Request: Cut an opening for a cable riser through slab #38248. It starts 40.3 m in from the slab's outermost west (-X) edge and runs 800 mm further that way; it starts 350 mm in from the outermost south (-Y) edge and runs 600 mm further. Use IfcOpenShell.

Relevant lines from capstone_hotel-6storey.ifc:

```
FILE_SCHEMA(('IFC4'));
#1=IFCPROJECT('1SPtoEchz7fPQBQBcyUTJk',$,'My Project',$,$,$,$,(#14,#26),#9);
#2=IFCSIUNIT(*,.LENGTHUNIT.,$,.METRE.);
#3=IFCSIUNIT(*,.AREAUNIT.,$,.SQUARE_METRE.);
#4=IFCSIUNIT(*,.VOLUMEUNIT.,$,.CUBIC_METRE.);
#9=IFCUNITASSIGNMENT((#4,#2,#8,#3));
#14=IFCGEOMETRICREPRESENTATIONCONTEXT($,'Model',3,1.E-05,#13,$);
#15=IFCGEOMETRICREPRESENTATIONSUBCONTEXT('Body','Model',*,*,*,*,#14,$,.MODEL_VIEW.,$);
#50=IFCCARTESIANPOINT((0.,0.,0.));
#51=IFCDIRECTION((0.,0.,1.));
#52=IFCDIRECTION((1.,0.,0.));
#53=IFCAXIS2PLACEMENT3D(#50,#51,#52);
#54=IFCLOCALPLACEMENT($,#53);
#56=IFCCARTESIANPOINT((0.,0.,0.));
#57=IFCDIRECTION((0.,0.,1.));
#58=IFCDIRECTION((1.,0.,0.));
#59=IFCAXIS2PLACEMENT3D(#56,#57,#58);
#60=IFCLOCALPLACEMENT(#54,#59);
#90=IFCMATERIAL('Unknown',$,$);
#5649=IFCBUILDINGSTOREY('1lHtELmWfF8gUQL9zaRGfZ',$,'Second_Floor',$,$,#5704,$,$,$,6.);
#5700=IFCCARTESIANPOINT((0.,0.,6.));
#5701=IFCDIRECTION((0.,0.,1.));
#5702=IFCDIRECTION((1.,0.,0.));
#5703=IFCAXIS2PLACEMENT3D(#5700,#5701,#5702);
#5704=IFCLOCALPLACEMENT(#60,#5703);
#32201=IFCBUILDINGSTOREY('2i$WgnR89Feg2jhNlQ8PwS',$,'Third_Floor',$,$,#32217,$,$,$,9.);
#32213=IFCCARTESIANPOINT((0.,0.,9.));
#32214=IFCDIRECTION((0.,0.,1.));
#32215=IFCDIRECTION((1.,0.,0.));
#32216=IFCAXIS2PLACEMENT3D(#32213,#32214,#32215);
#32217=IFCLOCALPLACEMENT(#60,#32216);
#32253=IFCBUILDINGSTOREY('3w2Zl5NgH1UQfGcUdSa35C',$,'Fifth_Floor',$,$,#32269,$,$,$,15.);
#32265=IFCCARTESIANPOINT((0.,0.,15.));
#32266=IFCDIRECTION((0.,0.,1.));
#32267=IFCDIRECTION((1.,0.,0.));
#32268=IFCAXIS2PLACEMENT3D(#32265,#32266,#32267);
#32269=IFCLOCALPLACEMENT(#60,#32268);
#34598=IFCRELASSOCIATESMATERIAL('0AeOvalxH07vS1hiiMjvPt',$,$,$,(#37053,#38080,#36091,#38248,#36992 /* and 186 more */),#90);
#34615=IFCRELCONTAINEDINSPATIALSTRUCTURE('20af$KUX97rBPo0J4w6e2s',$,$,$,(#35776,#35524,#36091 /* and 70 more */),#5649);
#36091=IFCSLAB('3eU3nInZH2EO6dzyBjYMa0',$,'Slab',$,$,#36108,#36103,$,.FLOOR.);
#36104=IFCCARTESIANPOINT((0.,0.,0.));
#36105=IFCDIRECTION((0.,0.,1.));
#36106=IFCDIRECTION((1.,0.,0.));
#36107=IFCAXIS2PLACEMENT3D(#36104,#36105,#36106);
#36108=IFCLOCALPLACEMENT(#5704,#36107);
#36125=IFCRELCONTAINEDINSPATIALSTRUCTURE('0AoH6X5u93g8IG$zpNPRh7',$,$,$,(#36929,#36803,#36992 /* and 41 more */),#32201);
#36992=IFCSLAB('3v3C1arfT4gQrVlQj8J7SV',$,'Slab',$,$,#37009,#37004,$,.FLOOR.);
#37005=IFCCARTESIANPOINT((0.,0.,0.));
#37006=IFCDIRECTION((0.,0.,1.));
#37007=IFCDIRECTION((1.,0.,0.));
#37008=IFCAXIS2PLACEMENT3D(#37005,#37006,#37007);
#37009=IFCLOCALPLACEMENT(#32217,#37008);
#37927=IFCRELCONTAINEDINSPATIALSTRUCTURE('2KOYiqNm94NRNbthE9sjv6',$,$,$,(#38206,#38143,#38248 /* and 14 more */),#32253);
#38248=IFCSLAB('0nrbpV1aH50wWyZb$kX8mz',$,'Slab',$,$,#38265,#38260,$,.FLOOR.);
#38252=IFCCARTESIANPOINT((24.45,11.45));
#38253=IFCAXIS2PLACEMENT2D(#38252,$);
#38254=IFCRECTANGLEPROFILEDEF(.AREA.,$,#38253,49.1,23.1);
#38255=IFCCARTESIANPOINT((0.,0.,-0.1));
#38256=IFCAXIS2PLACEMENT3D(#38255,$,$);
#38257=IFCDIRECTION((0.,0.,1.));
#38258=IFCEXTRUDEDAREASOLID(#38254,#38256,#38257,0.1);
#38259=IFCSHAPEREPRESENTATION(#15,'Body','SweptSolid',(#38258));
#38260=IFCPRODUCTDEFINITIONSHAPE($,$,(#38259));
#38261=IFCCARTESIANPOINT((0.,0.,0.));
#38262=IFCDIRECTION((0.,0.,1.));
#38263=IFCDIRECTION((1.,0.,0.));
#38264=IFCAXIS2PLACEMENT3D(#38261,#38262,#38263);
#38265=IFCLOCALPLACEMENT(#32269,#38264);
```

```python
import numpy as np
import ifcopenshell
import ifcopenshell.api.feature
import ifcopenshell.api.geometry
import ifcopenshell.api.root
import ifcopenshell.geom
import ifcopenshell.util.placement
import ifcopenshell.util.representation
import ifcopenshell.util.shape
import ifcopenshell.util.unit

model = ifcopenshell.open("capstone_hotel-6storey.ifc")
unit_scale = ifcopenshell.util.unit.calculate_unit_scale(model)
settings = ifcopenshell.geom.settings()


def volume(element):
    """Net volume in cubic metres, openings subtracted."""
    shape = ifcopenshell.geom.create_shape(settings, element)
    return ifcopenshell.util.shape.get_volume(shape.geometry)


slab = model.by_guid("0nrbpV1aH50wWyZb$kX8mz")
before = volume(slab)

# Extent in the slab's own axes, in metres. The edges named are its -X and -Y sides.
slab_shape = ifcopenshell.geom.create_shape(settings, slab)
vertices = ifcopenshell.util.shape.get_vertices(slab_shape.geometry)
x_min, y_min, bottom = vertices.min(axis=0)
top = vertices[:, 2].max()

opening = ifcopenshell.api.root.create_entity(model, ifc_class="IfcOpeningElement", name="Cable riser opening", predefined_type="OPENING")
context = ifcopenshell.util.representation.get_context(model, "Model", "Body", "MODEL_VIEW")
width, depth = 0.8, 0.6
outline = [(0.0, 0.0), (width, 0.0), (width, depth), (0.0, depth), (0.0, 0.0)]
# Overshoot both faces by 50 mm so the cut is clean.
shape = ifcopenshell.api.geometry.add_slab_representation(
    model, context=context, depth=top - bottom + 0.1, polyline=outline
)
ifcopenshell.api.geometry.assign_representation(model, product=opening, representation=shape)

matrix = ifcopenshell.util.placement.get_local_placement(slab.ObjectPlacement)
matrix[:, 3] = matrix @ np.append(np.array([x_min + 40.3, y_min + 0.35, bottom - 0.05]) / unit_scale, 1.0)
ifcopenshell.api.geometry.edit_object_placement(model, product=opening, matrix=matrix, is_si=False)
ifcopenshell.api.feature.add_feature(model, feature=opening, element=slab)

after = volume(slab)

print(f"slab volume {before:.3f} -> {after:.3f} m3")

model.write("capstone_hotel-6storey_v2.ifc")
```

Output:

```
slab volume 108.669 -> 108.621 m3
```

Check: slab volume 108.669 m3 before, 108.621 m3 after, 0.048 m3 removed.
